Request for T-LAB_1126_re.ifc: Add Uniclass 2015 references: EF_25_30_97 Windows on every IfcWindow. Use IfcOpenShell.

First a look at what the model holds.

```python
import ifcopenshell

model = ifcopenshell.open("T-LAB_1126_re.ifc")
print(model.schema)
print("classifications:", [c.Name for c in model.by_type("IfcClassification")])
for ifc_class in ("IfcDoor", "IfcRoof", "IfcStair", "IfcWall", "IfcWindow"):
    print(ifc_class, len(model.by_type(ifc_class)))
```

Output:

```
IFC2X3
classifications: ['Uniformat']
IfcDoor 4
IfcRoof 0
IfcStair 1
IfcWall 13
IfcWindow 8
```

```python
import ifcopenshell
import ifcopenshell.api.classification

model = ifcopenshell.open("T-LAB_1126_re.ifc")

# IFC2X3 requires Source and Edition and has no link from the project to the system.
system = model.create_entity("IfcClassification", Source="NBS", Edition="2015", Name="Uniclass 2015")

codes = {
    "IfcWindow": ("EF_25_30_97", "Windows"),
}
for ifc_class, (code, name) in codes.items():
    products = model.by_type(ifc_class)
    ifcopenshell.api.classification.add_reference(
        model, products=products, classification=system, identification=code, name=name
    )
    print(code, len(products))

model.write("T-LAB_1126_re_v2.ifc")
```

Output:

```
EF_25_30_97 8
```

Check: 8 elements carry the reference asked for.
